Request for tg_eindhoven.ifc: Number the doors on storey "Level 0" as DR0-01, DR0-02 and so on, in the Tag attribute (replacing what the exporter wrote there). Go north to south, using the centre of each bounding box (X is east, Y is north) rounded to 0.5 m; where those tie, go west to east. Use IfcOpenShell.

First a look at what the model holds.

```python
import ifcopenshell
import ifcopenshell.util.element
import ifcopenshell.util.placement

model = ifcopenshell.open("tg_eindhoven.ifc")
print(model.schema)
storey = next(s for s in model.by_type("IfcBuildingStorey") if s.Name == "Level 0")
doors = [e for e in ifcopenshell.util.element.get_decomposition(storey) if e.is_a("IfcDoor")]
for e in sorted(doors, key=lambda e: e.id()):
    origin = ifcopenshell.util.placement.get_local_placement(e.ObjectPlacement)[:3, 3]
    print(e.id(), e.Tag, e.Name, origin.round(2) + 0.0, sep=" | ")
```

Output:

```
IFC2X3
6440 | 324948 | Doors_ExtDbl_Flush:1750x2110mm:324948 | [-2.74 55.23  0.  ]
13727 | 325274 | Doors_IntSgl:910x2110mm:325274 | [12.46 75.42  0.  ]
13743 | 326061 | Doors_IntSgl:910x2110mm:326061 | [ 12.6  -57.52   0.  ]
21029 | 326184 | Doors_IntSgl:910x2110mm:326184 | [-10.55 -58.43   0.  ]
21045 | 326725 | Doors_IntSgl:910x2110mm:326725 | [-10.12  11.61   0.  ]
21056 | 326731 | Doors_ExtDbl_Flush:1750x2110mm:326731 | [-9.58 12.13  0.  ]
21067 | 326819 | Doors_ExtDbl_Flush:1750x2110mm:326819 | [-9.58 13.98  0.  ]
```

```python
import ifcopenshell
import ifcopenshell.geom
import ifcopenshell.util.element
import ifcopenshell.util.shape

model = ifcopenshell.open("tg_eindhoven.ifc")
settings = ifcopenshell.geom.settings()
settings.set("use-world-coords", True)


def centre(element):
    shape = ifcopenshell.geom.create_shape(settings, element)
    return ifcopenshell.util.shape.get_bbox_centroid(shape.geometry)


storey = next(s for s in model.by_type("IfcBuildingStorey") if s.Name == "Level 0")
doors = [e for e in ifcopenshell.util.element.get_decomposition(storey) if e.is_a("IfcDoor")]

# Insertion points can sit at a corner or the storey origin, so sort by the geometry (in metres).
centres = {e: centre(e) for e in doors}
doors.sort(key=lambda e: (-round(centres[e][1] / 0.5), centres[e][0]))

for i, e in enumerate(doors, start=1):
    number = f"DR0-{i:02d}"
    e.Tag = number
    print(e.id(), number)

model.write("tg_eindhoven_rev.ifc")
```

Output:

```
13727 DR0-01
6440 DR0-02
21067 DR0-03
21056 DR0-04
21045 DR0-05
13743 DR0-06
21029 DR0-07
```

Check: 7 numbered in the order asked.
